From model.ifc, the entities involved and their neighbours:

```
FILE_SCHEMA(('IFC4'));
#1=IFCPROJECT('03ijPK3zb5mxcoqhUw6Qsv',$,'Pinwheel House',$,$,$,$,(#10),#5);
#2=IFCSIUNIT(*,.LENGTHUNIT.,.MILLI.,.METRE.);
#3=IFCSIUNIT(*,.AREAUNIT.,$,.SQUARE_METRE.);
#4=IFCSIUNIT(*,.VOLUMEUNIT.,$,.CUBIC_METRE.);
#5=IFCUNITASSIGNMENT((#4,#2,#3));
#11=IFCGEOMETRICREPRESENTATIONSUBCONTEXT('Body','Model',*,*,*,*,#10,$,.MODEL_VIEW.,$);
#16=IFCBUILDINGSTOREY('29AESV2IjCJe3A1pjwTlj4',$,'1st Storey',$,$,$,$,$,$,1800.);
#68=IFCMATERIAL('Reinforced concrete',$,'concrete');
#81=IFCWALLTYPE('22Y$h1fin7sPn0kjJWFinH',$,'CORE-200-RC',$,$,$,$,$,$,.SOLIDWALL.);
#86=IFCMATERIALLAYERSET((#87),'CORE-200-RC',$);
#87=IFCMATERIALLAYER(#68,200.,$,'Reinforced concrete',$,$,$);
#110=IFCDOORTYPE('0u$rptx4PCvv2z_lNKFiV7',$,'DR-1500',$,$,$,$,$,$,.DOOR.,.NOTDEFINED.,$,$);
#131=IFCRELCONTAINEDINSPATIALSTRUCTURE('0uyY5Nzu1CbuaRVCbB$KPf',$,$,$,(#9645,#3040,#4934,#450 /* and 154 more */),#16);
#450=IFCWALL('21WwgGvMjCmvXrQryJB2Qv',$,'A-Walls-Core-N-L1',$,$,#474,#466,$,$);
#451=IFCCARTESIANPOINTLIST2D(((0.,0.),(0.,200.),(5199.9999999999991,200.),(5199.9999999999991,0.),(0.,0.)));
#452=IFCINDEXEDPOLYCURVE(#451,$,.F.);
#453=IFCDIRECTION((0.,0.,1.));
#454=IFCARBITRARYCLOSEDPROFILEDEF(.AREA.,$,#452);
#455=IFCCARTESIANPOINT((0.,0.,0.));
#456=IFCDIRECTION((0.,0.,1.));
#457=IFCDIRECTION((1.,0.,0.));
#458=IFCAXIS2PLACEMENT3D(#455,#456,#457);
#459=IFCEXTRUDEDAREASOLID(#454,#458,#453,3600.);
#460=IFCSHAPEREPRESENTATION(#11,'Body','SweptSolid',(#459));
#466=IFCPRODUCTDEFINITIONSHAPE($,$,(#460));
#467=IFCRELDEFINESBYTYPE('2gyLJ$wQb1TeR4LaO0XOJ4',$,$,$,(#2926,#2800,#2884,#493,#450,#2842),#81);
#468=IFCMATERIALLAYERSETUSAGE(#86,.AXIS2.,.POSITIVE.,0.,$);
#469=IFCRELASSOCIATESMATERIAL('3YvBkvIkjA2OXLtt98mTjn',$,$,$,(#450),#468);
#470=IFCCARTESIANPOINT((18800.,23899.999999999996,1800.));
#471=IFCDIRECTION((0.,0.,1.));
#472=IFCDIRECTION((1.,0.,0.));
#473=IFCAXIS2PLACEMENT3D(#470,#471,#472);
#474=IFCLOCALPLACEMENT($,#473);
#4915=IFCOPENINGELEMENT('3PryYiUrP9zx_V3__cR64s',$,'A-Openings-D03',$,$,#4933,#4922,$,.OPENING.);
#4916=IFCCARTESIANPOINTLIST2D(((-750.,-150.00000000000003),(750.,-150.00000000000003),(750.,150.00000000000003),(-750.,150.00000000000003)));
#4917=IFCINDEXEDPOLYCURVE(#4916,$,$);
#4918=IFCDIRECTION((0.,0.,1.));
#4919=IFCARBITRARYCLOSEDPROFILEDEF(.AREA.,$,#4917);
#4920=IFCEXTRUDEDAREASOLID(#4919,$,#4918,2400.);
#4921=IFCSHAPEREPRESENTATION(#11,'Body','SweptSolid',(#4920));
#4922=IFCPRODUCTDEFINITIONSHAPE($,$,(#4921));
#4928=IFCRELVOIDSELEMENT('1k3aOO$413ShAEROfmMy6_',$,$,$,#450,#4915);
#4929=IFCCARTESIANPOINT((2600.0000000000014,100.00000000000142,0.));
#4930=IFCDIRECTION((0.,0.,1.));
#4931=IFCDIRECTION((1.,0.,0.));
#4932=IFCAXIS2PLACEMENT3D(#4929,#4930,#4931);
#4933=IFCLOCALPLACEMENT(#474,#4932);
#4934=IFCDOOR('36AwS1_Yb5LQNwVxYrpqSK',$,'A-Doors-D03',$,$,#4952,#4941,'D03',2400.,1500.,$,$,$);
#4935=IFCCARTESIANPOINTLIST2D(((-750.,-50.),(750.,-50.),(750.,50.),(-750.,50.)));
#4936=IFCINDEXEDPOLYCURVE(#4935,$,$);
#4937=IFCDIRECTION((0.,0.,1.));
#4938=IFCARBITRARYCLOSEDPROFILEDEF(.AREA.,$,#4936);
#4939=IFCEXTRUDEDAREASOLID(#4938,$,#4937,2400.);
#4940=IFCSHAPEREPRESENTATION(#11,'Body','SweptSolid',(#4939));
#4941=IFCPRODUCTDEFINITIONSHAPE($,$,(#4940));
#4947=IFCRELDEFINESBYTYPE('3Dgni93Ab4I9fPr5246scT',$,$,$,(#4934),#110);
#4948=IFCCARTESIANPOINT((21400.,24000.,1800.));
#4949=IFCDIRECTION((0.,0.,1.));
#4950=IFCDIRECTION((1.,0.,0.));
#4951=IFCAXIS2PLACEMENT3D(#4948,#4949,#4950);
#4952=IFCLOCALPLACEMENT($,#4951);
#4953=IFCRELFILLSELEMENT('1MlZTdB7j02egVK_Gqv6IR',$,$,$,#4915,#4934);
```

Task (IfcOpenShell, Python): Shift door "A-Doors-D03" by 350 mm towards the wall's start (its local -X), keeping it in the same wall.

```python
import ifcopenshell
import ifcopenshell.api.geometry
import ifcopenshell.util.placement
import ifcopenshell.util.unit

model = ifcopenshell.open("model.ifc")
unit_scale = ifcopenshell.util.unit.calculate_unit_scale(model)

door = model.by_guid("36AwS1_Yb5LQNwVxYrpqSK")
opening = door.FillsVoids[0].RelatingOpeningElement
wall = opening.VoidsElements[0].RelatingBuildingElement

wall_matrix = ifcopenshell.util.placement.get_local_placement(wall.ObjectPlacement)
shift = wall_matrix[:3, 0] * -0.35 / unit_scale
before = ifcopenshell.util.placement.get_local_placement(door.ObjectPlacement)[:3, 3].copy()

# The door is not placed relative to its opening, so move both.
for product in (opening, door):
    matrix = ifcopenshell.util.placement.get_local_placement(product.ObjectPlacement)
    matrix[:3, 3] += shift
    ifcopenshell.api.geometry.edit_object_placement(model, product=product, matrix=matrix, is_si=False)

after = ifcopenshell.util.placement.get_local_placement(door.ObjectPlacement)[:3, 3]
print("door moved by", (after - before).round(3) + 0.0)

model.write("model_rev.ifc")
```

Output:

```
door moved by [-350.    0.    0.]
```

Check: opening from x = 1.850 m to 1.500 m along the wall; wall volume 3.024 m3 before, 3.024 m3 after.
